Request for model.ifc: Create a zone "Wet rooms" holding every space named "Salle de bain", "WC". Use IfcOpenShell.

First a look at what the model holds.

```python
import ifcopenshell

model = ifcopenshell.open("model.ifc")
print(model.schema)
seen = {}
for space in model.by_type("IfcSpace"):
    seen[space.LongName] = seen.get(space.LongName, 0) + 1
for name, count in sorted(seen.items(), key=str):
    print(count, "x", name)
print("zones:", [z.Name for z in model.by_type("IfcZone")][:20])
```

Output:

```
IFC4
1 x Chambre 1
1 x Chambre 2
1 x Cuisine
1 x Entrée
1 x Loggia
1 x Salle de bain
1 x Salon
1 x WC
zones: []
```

```python
import ifcopenshell
import ifcopenshell.api.group
import ifcopenshell.api.root

model = ifcopenshell.open("model.ifc")

names = {"Salle de bain", "WC"}
spaces = [s for s in model.by_type("IfcSpace") if s.LongName in names]

zone = ifcopenshell.api.root.create_entity(model, ifc_class="IfcZone", name="Wet rooms")
ifcopenshell.api.group.assign_group(model, products=spaces, group=zone)
print(len(spaces), "spaces in", zone.Name)

model.write("model_v2.ifc")
```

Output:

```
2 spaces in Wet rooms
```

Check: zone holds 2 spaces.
